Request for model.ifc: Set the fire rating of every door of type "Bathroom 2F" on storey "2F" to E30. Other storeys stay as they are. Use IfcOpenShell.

First a look at what the model holds.

```python
import ifcopenshell
import ifcopenshell.util.element

model = ifcopenshell.open("model.ifc")
print(model.schema)
storey = next(s for s in model.by_type("IfcBuildingStorey") if s.Name == "2F")
doors = [e for e in ifcopenshell.util.element.get_decomposition(storey) if e.is_a("IfcDoor")]
seen = {}
for e in doors:
    element_type = ifcopenshell.util.element.get_type(e)
    key = (element_type.Name if element_type != e and element_type else None, ifcopenshell.util.element.get_pset(e, "Pset_DoorCommon", "FireRating"))
    seen[key] = seen.get(key, 0) + 1
for (name, value), count in sorted(seen.items(), key=str):
    print(count, "x", name, "|", value)
```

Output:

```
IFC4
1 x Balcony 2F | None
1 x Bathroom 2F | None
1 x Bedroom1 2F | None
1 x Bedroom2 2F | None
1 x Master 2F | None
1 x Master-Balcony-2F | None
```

```python
import ifcopenshell
import ifcopenshell.api.pset
import ifcopenshell.util.element

model = ifcopenshell.open("model.ifc")

storey = next(s for s in model.by_type("IfcBuildingStorey") if s.Name == "2F")
doors = [e for e in ifcopenshell.util.element.get_decomposition(storey) if e.is_a("IfcDoor")]

count = 0
for e in doors:
    element_type = ifcopenshell.util.element.get_type(e)
    if element_type in (None, e) or element_type.Name != "Bathroom 2F":
        continue
    # add_pset returns the element's existing set when there is one.
    pset = ifcopenshell.api.pset.add_pset(model, product=e, name="Pset_DoorCommon")
    ifcopenshell.api.pset.edit_pset(model, pset=pset, properties={"FireRating": "E30"})
    count += 1

print(count, "doors updated")

model.write("model_updated.ifc")
```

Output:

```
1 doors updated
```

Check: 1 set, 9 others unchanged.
